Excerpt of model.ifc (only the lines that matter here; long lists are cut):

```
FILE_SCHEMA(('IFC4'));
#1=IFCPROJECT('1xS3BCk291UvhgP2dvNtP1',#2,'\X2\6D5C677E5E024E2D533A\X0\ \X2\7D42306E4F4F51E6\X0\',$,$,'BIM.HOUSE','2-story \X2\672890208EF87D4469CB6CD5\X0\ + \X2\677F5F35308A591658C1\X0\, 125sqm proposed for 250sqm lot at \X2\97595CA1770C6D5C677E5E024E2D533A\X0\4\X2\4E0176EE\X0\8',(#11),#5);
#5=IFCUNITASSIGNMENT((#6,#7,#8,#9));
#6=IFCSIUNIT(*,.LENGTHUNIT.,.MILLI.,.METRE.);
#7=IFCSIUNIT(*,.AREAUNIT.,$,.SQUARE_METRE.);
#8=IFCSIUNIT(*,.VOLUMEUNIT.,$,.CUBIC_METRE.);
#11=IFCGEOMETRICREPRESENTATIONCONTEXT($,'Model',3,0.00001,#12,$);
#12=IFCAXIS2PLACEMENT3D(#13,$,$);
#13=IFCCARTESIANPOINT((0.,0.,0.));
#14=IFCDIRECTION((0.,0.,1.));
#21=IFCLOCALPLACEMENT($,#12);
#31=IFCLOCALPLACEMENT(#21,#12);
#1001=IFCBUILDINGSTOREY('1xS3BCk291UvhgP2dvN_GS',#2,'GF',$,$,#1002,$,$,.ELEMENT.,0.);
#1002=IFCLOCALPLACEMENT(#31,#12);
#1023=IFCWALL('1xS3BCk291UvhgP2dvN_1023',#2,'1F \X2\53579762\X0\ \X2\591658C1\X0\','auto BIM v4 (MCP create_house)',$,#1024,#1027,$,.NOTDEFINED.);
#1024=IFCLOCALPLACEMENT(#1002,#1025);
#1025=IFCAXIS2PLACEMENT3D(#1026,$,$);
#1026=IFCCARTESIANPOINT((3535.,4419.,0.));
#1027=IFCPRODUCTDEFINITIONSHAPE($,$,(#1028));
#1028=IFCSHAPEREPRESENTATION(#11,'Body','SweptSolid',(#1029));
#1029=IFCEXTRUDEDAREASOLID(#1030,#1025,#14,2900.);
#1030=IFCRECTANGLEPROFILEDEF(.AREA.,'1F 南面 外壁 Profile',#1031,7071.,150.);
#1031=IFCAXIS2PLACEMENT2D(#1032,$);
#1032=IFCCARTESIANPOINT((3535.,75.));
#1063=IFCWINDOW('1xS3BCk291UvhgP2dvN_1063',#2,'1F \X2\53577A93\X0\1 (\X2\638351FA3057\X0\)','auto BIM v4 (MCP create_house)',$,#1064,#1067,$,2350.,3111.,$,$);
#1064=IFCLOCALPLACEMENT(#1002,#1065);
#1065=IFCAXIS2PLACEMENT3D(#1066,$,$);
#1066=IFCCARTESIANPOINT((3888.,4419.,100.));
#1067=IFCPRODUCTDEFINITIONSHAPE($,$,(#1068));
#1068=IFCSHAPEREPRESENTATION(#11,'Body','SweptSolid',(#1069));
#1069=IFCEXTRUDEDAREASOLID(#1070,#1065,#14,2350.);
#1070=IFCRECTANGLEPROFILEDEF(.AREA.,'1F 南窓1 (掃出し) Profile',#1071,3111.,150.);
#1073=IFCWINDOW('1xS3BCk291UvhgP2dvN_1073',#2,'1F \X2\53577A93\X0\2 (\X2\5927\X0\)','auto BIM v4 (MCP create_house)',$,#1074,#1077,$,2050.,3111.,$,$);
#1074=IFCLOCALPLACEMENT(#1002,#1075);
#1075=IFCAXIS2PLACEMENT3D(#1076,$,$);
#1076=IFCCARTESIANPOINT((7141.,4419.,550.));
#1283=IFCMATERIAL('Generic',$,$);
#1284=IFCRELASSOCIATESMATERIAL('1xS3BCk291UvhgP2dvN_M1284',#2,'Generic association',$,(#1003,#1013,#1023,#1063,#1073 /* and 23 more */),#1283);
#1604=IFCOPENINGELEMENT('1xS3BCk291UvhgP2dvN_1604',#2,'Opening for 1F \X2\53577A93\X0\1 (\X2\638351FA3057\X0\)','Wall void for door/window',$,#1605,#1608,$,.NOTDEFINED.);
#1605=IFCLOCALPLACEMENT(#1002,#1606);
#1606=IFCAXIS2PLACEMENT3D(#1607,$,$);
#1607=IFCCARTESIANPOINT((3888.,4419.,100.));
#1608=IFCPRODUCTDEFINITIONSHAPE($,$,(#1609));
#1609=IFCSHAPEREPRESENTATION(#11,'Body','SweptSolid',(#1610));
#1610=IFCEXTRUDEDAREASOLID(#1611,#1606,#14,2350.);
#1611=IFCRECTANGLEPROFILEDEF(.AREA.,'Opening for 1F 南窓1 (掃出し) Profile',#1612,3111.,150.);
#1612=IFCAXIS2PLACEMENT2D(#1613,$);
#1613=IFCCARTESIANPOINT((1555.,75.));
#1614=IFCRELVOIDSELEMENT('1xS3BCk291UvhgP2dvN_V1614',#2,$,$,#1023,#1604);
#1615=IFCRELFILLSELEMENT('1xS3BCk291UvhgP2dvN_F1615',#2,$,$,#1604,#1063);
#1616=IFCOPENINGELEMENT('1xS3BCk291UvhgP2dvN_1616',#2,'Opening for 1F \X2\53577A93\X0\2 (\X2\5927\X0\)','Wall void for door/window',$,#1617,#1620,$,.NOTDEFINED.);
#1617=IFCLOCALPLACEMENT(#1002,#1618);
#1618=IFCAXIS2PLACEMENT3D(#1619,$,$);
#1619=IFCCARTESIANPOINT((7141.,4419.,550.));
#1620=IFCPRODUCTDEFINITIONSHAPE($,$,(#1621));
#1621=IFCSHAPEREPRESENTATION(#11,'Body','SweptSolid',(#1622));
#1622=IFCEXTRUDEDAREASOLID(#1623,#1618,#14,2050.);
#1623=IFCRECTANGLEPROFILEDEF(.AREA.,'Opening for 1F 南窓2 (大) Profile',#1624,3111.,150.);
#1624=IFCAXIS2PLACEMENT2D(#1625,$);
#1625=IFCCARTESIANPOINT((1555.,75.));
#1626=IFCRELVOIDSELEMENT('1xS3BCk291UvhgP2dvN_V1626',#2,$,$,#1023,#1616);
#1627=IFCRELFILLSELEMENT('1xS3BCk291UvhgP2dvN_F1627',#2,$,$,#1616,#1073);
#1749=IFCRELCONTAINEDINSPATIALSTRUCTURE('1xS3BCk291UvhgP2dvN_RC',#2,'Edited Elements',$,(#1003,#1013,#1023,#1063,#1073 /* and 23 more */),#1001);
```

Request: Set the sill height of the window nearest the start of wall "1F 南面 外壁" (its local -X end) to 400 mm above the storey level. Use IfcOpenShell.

```python
import numpy as np
import ifcopenshell
import ifcopenshell.api.geometry
import ifcopenshell.geom
import ifcopenshell.util.element
import ifcopenshell.util.placement
import ifcopenshell.util.shape
import ifcopenshell.util.unit

model = ifcopenshell.open("model.ifc")
unit_scale = ifcopenshell.util.unit.calculate_unit_scale(model)

window = model.by_id(1063)
opening = window.FillsVoids[0].RelatingOpeningElement
storey = ifcopenshell.util.element.get_container(window, ifc_class="IfcBuildingStorey")
level = ifcopenshell.util.placement.get_local_placement(storey.ObjectPlacement)[2, 3]

# The opening's origin need not be at the sill, so measure its lowest point.
shape = ifcopenshell.geom.create_shape(ifcopenshell.geom.settings(), opening)
bottom = ifcopenshell.util.shape.get_shape_bottom_elevation(shape, shape.geometry) / unit_scale
dz = level + 400.0 - bottom

shift = np.array([0.0, 0.0, dz])
# The window is not placed relative to its opening, so move both.
for product in (opening, window):
    matrix = ifcopenshell.util.placement.get_local_placement(product.ObjectPlacement)
    matrix[:3, 3] += shift
    ifcopenshell.api.geometry.edit_object_placement(model, product=product, matrix=matrix, is_si=False)

print(f"moved by {dz * unit_scale:+.3f} m")

model.write("model-out.ifc")
```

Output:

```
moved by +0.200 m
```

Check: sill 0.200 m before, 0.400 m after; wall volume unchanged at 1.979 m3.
